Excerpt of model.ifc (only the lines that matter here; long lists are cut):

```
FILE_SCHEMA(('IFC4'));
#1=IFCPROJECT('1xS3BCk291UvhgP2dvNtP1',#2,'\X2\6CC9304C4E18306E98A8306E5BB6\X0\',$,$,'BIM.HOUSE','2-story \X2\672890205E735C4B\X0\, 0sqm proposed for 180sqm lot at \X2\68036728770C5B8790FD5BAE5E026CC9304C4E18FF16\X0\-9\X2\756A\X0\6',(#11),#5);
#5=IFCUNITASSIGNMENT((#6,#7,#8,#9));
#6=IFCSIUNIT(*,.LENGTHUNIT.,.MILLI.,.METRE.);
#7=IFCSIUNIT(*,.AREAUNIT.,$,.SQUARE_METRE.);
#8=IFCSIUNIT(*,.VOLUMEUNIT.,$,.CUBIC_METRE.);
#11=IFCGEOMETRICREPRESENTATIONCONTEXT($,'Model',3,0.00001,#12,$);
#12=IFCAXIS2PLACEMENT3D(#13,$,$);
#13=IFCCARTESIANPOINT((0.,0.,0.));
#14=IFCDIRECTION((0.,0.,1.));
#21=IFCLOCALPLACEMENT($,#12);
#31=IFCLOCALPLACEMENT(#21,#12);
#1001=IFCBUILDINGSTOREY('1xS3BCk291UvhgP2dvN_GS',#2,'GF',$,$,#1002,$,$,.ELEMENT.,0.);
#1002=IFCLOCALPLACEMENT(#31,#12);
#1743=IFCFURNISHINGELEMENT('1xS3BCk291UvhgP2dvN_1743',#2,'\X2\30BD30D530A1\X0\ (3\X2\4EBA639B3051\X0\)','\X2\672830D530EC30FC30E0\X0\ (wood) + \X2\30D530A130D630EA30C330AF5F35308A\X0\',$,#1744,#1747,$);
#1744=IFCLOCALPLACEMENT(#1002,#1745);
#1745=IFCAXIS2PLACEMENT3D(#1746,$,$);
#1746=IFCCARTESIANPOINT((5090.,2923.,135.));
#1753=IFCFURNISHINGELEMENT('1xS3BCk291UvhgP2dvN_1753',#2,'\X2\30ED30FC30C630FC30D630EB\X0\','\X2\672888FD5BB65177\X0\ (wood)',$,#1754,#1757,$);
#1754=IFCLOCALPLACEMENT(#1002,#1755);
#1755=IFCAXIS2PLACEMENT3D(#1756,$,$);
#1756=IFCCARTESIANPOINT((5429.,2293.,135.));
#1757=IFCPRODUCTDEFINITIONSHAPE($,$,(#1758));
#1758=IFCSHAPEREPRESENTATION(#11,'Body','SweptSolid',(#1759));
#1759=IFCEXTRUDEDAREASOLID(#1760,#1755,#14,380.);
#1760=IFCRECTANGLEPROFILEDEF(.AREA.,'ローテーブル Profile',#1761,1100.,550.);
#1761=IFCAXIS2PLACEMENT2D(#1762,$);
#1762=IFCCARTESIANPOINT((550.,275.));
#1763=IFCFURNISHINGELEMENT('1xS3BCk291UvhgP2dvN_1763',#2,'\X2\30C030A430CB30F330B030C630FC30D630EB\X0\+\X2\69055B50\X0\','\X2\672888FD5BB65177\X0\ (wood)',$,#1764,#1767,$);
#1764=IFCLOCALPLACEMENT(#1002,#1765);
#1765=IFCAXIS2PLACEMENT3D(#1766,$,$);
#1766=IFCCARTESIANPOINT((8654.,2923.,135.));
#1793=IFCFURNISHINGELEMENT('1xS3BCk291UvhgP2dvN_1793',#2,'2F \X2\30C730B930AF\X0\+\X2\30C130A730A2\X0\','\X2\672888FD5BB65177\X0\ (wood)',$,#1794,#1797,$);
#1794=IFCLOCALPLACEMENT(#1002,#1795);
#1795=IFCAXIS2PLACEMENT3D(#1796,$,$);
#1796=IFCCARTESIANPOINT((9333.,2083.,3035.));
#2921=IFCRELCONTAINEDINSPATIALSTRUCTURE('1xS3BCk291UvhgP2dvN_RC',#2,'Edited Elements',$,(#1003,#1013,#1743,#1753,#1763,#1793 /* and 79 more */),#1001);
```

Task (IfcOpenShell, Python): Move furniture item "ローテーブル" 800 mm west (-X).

```python
import ifcopenshell
import ifcopenshell.api.geometry
import ifcopenshell.util.placement

model = ifcopenshell.open("model.ifc")

item = model.by_guid("1xS3BCk291UvhgP2dvN_1753")
matrix = ifcopenshell.util.placement.get_local_placement(item.ObjectPlacement)
matrix[0, 3] -= 800.0
ifcopenshell.api.geometry.edit_object_placement(model, product=item, matrix=matrix, is_si=False)

print(ifcopenshell.util.placement.get_local_placement(item.ObjectPlacement).round(3) + 0.0)

model.write("model_rev.ifc")
```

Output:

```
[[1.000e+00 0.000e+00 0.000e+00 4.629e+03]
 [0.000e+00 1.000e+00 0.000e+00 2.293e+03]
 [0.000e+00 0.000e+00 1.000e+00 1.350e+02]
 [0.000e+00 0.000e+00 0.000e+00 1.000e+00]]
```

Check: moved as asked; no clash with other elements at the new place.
